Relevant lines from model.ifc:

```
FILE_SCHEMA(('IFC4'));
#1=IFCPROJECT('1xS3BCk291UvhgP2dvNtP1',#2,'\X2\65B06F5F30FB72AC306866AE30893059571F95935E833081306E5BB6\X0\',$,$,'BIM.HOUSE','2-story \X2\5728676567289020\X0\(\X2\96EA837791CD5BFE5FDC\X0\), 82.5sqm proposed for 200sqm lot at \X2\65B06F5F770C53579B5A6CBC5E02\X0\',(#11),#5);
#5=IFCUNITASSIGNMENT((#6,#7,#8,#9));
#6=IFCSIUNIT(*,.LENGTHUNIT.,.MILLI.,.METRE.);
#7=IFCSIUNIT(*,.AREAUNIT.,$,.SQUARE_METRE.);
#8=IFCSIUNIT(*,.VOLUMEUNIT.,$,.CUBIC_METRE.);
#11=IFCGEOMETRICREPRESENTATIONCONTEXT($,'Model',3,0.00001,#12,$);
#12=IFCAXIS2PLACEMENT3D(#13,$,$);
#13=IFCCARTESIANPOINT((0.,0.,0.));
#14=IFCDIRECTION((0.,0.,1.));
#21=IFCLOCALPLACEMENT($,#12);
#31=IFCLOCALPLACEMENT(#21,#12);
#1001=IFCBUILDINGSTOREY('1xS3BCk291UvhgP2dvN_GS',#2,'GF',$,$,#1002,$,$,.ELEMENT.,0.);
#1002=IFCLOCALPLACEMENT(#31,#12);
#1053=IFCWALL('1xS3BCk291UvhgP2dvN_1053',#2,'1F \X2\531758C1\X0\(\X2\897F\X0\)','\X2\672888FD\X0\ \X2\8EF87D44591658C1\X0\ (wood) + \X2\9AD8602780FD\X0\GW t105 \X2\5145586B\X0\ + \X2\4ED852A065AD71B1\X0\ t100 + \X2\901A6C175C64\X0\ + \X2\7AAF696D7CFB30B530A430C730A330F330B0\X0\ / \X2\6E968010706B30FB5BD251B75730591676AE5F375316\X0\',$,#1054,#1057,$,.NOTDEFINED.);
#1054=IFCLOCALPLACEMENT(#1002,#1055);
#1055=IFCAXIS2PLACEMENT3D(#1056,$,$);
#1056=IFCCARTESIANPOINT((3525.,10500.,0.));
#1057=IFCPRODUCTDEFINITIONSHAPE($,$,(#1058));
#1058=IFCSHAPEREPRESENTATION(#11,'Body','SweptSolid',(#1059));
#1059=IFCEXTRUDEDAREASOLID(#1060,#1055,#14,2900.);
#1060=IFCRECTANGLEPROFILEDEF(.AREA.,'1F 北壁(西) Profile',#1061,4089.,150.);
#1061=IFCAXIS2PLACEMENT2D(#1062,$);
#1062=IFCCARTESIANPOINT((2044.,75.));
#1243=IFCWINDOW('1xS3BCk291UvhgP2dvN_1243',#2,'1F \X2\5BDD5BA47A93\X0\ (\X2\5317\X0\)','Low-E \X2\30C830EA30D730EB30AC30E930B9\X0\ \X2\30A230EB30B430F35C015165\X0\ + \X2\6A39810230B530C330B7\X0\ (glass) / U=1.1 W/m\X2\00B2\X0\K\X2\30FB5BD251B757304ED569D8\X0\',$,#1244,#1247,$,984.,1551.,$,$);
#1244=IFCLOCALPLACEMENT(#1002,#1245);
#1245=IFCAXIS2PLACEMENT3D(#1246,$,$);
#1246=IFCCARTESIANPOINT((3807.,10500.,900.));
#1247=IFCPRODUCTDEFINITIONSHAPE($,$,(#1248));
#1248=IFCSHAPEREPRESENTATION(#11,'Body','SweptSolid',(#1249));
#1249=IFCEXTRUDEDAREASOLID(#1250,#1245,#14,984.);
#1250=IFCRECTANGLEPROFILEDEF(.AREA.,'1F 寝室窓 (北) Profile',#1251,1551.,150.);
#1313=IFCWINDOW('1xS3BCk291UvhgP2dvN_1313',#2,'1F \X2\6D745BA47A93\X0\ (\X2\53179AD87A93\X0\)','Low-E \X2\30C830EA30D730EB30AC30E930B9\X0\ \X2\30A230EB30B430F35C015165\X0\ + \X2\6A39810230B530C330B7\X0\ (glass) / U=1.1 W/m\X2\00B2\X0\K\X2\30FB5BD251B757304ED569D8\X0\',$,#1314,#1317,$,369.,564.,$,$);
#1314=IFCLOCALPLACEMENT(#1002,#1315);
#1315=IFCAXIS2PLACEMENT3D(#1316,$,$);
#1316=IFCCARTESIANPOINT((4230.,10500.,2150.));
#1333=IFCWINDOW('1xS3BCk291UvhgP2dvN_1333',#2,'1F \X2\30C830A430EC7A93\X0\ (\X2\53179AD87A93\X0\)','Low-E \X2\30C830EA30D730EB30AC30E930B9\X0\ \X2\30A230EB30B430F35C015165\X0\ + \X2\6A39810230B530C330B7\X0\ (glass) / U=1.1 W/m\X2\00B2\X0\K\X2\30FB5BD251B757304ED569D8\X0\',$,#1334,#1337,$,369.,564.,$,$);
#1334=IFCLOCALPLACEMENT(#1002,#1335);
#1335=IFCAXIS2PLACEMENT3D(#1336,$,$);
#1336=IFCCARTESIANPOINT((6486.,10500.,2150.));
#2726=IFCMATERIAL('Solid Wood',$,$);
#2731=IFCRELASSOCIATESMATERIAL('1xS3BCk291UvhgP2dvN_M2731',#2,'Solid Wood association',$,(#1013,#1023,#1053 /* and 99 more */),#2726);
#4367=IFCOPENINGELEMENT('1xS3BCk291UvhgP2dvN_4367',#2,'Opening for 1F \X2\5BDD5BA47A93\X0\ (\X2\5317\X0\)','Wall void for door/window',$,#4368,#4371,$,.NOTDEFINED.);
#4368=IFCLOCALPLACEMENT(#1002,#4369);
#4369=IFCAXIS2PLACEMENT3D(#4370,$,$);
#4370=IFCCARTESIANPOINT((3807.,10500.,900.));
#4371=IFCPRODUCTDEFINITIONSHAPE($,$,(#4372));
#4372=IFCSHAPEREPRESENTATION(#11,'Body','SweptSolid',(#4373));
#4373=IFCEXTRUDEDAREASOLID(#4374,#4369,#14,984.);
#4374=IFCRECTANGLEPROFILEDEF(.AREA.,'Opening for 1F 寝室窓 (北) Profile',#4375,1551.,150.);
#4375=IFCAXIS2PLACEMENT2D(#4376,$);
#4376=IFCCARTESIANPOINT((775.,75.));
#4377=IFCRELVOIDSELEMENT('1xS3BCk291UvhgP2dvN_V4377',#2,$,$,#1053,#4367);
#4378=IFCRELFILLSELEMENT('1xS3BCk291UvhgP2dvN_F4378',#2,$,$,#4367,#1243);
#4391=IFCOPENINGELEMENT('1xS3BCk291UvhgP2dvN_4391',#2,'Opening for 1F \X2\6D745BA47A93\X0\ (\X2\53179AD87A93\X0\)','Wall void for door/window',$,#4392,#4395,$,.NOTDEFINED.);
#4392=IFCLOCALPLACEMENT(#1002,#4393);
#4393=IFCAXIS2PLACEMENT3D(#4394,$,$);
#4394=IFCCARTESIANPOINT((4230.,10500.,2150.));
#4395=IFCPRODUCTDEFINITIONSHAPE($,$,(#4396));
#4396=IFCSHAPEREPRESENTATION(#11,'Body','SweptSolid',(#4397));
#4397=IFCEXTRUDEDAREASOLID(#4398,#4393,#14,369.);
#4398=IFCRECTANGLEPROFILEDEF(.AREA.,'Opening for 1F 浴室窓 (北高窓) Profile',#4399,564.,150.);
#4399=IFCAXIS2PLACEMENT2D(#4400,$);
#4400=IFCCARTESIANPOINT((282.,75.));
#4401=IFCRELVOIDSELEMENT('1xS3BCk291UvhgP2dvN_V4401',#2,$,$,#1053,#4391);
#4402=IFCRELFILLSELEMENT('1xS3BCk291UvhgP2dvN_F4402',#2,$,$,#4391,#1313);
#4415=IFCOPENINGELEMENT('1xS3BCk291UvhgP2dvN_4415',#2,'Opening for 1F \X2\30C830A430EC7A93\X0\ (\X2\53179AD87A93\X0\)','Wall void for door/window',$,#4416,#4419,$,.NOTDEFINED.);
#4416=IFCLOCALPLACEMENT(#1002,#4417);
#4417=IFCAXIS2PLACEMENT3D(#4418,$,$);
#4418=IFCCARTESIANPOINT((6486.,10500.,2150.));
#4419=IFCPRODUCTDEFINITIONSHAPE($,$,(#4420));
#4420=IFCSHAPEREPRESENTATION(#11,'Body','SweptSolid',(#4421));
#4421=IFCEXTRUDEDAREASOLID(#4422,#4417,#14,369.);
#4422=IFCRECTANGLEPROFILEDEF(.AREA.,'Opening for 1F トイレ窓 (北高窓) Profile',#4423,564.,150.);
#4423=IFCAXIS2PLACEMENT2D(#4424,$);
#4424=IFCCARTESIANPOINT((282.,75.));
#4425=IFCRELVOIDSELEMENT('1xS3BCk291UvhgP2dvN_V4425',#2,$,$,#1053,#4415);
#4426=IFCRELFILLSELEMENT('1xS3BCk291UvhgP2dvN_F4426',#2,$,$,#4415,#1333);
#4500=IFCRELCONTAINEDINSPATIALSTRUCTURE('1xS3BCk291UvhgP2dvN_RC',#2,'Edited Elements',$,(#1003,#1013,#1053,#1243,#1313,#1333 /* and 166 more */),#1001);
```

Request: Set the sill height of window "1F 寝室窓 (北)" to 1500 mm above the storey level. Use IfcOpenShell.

```python
import numpy as np
import ifcopenshell
import ifcopenshell.api.geometry
import ifcopenshell.geom
import ifcopenshell.util.element
import ifcopenshell.util.placement
import ifcopenshell.util.shape
import ifcopenshell.util.unit

model = ifcopenshell.open("model.ifc")
unit_scale = ifcopenshell.util.unit.calculate_unit_scale(model)

window = model.by_guid("1xS3BCk291UvhgP2dvN_1243")
opening = window.FillsVoids[0].RelatingOpeningElement
storey = ifcopenshell.util.element.get_container(window, ifc_class="IfcBuildingStorey")
level = ifcopenshell.util.placement.get_local_placement(storey.ObjectPlacement)[2, 3]

# The opening's origin need not be at the sill, so measure its lowest point.
shape = ifcopenshell.geom.create_shape(ifcopenshell.geom.settings(), opening)
bottom = ifcopenshell.util.shape.get_shape_bottom_elevation(shape, shape.geometry) / unit_scale
dz = level + 1.5 / unit_scale - bottom

shift = np.array([0.0, 0.0, dz])
# The window is not placed relative to its opening, so move both.
for product in (opening, window):
    matrix = ifcopenshell.util.placement.get_local_placement(product.ObjectPlacement)
    matrix[:3, 3] += shift
    ifcopenshell.api.geometry.edit_object_placement(model, product=product, matrix=matrix, is_si=False)

print(f"moved by {dz * unit_scale:+.3f} m")

model.write("model_edited.ifc")
```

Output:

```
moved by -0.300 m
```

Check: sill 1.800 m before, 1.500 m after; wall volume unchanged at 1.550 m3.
